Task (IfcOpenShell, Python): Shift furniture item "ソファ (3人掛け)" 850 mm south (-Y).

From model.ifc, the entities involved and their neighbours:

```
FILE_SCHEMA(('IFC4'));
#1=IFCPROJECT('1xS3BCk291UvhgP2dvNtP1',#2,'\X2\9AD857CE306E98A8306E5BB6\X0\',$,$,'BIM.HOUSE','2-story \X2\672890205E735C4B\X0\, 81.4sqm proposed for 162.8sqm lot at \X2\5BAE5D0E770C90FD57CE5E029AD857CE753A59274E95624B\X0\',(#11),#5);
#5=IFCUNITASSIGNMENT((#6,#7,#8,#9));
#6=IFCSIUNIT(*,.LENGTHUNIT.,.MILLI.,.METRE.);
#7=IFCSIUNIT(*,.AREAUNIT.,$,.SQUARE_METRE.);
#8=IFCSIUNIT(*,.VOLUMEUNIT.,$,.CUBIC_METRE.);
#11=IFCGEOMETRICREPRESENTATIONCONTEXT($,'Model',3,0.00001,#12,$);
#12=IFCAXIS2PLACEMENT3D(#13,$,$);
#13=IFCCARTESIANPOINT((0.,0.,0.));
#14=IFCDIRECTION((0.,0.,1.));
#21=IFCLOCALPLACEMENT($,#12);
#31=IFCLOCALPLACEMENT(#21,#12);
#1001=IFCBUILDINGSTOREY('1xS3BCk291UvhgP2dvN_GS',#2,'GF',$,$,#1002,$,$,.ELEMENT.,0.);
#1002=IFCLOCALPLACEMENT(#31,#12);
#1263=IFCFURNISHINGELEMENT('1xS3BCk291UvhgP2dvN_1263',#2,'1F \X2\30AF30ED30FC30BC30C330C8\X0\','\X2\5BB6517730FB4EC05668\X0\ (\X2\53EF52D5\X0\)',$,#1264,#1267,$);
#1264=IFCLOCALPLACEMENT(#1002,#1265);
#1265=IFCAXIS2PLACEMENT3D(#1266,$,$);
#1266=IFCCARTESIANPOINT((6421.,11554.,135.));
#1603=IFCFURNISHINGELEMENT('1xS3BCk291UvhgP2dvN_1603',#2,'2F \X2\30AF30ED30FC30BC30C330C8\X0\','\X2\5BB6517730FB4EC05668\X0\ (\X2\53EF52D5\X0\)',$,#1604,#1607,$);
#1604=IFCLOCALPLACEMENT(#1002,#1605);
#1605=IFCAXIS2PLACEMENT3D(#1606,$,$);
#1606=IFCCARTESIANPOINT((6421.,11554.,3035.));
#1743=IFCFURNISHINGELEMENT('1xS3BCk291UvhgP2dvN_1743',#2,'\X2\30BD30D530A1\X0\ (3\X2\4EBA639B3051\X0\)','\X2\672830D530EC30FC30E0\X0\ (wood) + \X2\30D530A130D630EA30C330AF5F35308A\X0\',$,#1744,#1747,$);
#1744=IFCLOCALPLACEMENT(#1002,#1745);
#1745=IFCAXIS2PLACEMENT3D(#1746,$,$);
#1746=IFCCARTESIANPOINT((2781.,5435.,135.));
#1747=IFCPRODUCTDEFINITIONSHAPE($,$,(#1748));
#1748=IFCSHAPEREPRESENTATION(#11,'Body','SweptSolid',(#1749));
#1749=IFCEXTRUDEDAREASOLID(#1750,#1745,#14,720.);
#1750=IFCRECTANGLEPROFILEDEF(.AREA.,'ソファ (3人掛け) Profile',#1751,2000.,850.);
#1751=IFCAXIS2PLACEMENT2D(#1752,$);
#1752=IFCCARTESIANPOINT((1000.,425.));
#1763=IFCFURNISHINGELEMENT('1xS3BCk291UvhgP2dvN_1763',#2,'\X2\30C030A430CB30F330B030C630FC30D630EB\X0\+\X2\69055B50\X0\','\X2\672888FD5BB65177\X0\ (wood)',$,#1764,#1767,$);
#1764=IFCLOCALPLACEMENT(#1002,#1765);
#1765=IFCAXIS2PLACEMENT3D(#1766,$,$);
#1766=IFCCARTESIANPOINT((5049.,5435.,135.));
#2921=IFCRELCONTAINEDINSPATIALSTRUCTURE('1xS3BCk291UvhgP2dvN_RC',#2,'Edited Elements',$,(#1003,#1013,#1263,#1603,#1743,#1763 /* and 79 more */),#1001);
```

```python
import ifcopenshell
import ifcopenshell.api.geometry
import ifcopenshell.util.placement
import ifcopenshell.util.unit

model = ifcopenshell.open("model.ifc")
unit_scale = ifcopenshell.util.unit.calculate_unit_scale(model)

item = model.by_guid("1xS3BCk291UvhgP2dvN_1743")
matrix = ifcopenshell.util.placement.get_local_placement(item.ObjectPlacement)
matrix[1, 3] -= 0.85 / unit_scale
ifcopenshell.api.geometry.edit_object_placement(model, product=item, matrix=matrix, is_si=False)

print(ifcopenshell.util.placement.get_local_placement(item.ObjectPlacement).round(3) + 0.0)

model.write("model_v2.ifc")
```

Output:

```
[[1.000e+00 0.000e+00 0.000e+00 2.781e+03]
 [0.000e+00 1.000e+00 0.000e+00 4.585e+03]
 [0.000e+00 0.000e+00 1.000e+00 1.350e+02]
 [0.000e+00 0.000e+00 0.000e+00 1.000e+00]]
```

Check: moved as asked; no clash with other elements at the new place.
